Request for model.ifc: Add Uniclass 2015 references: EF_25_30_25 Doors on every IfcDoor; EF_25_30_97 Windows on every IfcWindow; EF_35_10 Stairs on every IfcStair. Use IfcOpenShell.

First a look at what the model holds.

```python
import ifcopenshell

model = ifcopenshell.open("model.ifc")
print(model.schema)
print("classifications:", [c.Name for c in model.by_type("IfcClassification")])
for ifc_class in ("IfcDoor", "IfcRoof", "IfcStair", "IfcWall", "IfcWindow"):
    print(ifc_class, len(model.by_type(ifc_class)))
```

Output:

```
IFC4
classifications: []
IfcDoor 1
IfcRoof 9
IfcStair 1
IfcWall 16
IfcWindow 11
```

```python
import ifcopenshell
import ifcopenshell.api.classification

model = ifcopenshell.open("model.ifc")

system = ifcopenshell.api.classification.add_classification(model, classification="Uniclass 2015")

codes = {
    "IfcDoor": ("EF_25_30_25", "Doors"),
    "IfcWindow": ("EF_25_30_97", "Windows"),
    "IfcStair": ("EF_35_10", "Stairs"),
}
for ifc_class, (code, name) in codes.items():
    products = model.by_type(ifc_class)
    ifcopenshell.api.classification.add_reference(
        model, products=products, classification=system, identification=code, name=name
    )
    print(code, len(products))

model.write("model_edited.ifc")
```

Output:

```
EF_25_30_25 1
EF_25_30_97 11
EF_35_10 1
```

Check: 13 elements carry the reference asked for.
